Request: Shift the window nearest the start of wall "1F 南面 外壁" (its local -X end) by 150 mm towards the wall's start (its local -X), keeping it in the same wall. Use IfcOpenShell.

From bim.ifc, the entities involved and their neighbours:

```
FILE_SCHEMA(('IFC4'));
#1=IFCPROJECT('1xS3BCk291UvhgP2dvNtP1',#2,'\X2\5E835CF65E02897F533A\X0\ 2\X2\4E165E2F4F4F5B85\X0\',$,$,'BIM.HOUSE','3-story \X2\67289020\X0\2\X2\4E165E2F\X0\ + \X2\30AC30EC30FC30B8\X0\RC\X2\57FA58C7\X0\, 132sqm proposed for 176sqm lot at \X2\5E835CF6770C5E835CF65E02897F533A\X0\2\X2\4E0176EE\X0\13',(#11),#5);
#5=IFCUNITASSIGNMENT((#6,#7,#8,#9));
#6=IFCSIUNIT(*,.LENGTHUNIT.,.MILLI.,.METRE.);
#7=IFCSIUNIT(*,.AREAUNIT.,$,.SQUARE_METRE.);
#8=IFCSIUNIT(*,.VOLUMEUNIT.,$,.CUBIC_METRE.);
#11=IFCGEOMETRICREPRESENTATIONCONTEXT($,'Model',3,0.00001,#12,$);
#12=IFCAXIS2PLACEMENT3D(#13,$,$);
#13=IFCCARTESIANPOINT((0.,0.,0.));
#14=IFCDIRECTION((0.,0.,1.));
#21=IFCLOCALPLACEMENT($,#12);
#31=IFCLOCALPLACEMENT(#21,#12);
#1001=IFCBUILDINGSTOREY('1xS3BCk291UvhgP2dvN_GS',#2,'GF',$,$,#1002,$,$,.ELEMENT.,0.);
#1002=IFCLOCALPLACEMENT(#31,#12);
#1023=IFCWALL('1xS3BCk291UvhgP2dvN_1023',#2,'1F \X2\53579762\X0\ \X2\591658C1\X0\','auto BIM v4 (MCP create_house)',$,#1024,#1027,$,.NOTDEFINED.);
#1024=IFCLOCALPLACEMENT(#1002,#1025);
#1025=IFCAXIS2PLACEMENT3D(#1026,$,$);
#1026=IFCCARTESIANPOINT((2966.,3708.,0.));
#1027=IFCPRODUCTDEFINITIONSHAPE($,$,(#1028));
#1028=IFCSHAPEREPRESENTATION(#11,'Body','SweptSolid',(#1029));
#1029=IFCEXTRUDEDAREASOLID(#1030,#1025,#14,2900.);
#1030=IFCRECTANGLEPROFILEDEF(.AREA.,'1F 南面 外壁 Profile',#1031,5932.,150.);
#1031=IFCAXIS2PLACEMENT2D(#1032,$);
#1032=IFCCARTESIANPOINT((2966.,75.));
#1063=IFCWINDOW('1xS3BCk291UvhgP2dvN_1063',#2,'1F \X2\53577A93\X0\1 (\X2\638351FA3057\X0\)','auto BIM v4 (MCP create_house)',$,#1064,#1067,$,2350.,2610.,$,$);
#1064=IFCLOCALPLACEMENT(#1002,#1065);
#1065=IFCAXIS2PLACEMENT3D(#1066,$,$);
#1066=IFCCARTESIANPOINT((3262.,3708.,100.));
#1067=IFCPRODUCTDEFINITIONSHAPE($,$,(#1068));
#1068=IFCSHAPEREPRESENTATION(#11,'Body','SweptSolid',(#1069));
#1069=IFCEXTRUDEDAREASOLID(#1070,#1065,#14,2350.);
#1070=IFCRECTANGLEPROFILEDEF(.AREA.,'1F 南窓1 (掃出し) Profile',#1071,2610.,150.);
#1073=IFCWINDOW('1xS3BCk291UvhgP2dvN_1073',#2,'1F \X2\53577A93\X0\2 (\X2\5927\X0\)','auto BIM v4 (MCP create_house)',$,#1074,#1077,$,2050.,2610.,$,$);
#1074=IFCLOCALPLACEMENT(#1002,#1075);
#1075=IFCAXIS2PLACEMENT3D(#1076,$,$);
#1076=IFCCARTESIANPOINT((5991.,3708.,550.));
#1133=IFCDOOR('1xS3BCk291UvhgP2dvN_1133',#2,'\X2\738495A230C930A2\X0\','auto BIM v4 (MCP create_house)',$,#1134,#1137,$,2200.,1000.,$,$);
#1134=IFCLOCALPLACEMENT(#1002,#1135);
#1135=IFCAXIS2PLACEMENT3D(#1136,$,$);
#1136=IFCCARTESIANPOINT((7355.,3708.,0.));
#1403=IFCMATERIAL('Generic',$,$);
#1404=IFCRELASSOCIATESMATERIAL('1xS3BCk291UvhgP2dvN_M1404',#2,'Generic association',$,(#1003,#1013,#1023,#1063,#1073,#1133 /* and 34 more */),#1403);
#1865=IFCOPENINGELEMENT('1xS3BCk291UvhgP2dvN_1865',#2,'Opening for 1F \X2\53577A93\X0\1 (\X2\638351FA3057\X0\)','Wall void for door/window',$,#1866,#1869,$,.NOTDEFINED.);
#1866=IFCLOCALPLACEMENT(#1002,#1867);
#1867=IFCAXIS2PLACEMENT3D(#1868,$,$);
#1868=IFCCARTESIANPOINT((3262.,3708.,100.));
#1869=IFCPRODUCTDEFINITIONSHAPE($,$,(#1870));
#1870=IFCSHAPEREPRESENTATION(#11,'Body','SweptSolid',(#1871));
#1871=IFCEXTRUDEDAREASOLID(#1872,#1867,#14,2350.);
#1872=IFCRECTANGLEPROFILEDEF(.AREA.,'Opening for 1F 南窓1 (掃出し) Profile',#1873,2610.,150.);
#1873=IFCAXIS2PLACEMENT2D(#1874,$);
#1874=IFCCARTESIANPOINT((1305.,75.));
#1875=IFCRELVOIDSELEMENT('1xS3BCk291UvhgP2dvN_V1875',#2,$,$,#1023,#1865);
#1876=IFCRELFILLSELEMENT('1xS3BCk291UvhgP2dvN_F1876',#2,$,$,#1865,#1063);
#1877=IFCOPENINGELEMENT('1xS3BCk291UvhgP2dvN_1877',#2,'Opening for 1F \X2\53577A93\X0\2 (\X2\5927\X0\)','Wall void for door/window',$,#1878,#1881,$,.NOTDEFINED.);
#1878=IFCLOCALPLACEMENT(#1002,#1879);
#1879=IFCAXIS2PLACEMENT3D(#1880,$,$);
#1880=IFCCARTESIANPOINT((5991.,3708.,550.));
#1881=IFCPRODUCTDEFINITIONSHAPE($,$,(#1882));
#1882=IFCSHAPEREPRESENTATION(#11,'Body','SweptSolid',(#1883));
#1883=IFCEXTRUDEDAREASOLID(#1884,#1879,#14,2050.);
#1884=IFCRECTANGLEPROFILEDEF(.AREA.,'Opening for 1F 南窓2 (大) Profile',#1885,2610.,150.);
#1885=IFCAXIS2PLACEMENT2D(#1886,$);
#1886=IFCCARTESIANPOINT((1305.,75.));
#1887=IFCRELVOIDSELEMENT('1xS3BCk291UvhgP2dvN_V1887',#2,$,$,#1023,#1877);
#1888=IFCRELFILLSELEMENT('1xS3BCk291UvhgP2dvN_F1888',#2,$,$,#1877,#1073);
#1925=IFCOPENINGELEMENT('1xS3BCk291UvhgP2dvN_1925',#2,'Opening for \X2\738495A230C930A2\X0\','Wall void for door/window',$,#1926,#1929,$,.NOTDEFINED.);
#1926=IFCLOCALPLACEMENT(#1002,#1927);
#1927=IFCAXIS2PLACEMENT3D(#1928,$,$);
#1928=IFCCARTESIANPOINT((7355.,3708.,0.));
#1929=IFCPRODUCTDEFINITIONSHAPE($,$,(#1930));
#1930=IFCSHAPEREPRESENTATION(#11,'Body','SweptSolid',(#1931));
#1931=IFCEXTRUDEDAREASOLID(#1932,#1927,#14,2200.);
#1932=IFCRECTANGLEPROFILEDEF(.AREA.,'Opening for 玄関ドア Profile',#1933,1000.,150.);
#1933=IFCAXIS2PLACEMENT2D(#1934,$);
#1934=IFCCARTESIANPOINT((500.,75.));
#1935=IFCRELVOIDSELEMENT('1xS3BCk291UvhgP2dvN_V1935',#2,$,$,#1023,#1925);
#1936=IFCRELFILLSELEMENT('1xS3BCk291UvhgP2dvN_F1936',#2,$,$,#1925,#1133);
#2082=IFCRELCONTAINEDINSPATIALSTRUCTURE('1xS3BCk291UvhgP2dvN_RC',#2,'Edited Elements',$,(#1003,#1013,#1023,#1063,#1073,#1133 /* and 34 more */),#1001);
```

```python
import ifcopenshell
import ifcopenshell.api.geometry
import ifcopenshell.util.placement

model = ifcopenshell.open("bim.ifc")

window = model.by_guid("1xS3BCk291UvhgP2dvN_1063")
opening = window.FillsVoids[0].RelatingOpeningElement
wall = opening.VoidsElements[0].RelatingBuildingElement

wall_matrix = ifcopenshell.util.placement.get_local_placement(wall.ObjectPlacement)
shift = wall_matrix[:3, 0] * -150.0
before = ifcopenshell.util.placement.get_local_placement(window.ObjectPlacement)[:3, 3].copy()

# The window is not placed relative to its opening, so move both.
for product in (opening, window):
    matrix = ifcopenshell.util.placement.get_local_placement(product.ObjectPlacement)
    matrix[:3, 3] += shift
    ifcopenshell.api.geometry.edit_object_placement(model, product=product, matrix=matrix, is_si=False)

after = ifcopenshell.util.placement.get_local_placement(window.ObjectPlacement)[:3, 3]
print("window moved by", (after - before).round(3) + 0.0)

model.write("bim_v2.ifc")
```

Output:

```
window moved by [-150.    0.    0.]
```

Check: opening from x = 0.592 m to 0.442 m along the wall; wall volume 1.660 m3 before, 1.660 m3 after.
